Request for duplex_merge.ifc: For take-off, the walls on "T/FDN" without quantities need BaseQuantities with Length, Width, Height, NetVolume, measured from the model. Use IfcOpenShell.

First a look at what the model holds.

```python
import ifcopenshell
import ifcopenshell.util.element
import ifcopenshell.util.unit

model = ifcopenshell.open("duplex_merge.ifc")
print(model.schema)
for unit_type in ("LENGTHUNIT", "AREAUNIT", "VOLUMEUNIT"):
    print(unit_type, ifcopenshell.util.unit.calculate_unit_scale(model, unit_type))
storey = next(s for s in model.by_type("IfcBuildingStorey") if s.Name == "T/FDN")
walls = [e for e in ifcopenshell.util.element.get_decomposition(storey) if e.is_a("IfcWall")]
for e in sorted(walls, key=lambda e: e.id()):
    print(e.id(), e.is_a(), e.Name, list(ifcopenshell.util.element.get_psets(e, qtos_only=True)), sep=" | ")
```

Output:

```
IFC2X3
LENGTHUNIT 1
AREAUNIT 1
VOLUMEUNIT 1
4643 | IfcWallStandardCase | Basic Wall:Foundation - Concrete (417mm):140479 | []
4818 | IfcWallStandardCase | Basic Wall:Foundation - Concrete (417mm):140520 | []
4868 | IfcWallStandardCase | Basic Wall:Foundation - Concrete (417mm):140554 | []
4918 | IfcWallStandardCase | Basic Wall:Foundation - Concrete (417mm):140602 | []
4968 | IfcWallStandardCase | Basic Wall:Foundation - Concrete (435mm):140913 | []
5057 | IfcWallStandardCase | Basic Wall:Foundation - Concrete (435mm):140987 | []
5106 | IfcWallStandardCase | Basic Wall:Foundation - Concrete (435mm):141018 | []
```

```python
import ifcopenshell
import ifcopenshell.api.pset
import ifcopenshell.geom
import ifcopenshell.util.element
import ifcopenshell.util.shape
import ifcopenshell.util.unit

model = ifcopenshell.open("duplex_merge.ifc")
unit_scale = ifcopenshell.util.unit.calculate_unit_scale(model)
volume_scale = ifcopenshell.util.unit.calculate_unit_scale(model, "VOLUMEUNIT")
settings = ifcopenshell.geom.settings()

storey = next(s for s in model.by_type("IfcBuildingStorey") if s.Name == "T/FDN")
walls = [e for e in ifcopenshell.util.element.get_decomposition(storey) if e.is_a("IfcWall")]

for e in sorted(walls, key=lambda e: e.id()):
    if ifcopenshell.util.element.get_psets(e, qtos_only=True, should_inherit=False):
        continue
    # Geometry comes back in metres, in the element's own axes.
    shape = ifcopenshell.geom.create_shape(settings, e)
    values = {
        "Length": ifcopenshell.util.shape.get_x(shape.geometry) / unit_scale,
        "Width": ifcopenshell.util.shape.get_y(shape.geometry) / unit_scale,
        "Height": ifcopenshell.util.shape.get_z(shape.geometry) / unit_scale,
        "NetVolume": ifcopenshell.util.shape.get_volume(shape.geometry) / volume_scale,
    }
    qto = ifcopenshell.api.pset.add_qto(model, product=e, name="BaseQuantities")
    ifcopenshell.api.pset.edit_qto(model, qto=qto, properties=values)
    print(e.id(), {k: round(v, 3) for k, v in values.items()})

model.write("duplex_merge_edited.ifc")
```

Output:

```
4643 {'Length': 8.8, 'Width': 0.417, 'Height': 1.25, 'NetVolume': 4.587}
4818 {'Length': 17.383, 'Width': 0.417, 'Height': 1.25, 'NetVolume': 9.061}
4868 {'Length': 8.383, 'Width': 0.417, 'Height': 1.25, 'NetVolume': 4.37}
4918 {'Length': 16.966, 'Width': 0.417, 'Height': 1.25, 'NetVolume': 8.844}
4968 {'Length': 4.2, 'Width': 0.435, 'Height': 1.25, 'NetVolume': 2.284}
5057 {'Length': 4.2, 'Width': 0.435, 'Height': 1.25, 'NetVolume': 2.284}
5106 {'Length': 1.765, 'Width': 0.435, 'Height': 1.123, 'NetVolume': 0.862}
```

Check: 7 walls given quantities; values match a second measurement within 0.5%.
